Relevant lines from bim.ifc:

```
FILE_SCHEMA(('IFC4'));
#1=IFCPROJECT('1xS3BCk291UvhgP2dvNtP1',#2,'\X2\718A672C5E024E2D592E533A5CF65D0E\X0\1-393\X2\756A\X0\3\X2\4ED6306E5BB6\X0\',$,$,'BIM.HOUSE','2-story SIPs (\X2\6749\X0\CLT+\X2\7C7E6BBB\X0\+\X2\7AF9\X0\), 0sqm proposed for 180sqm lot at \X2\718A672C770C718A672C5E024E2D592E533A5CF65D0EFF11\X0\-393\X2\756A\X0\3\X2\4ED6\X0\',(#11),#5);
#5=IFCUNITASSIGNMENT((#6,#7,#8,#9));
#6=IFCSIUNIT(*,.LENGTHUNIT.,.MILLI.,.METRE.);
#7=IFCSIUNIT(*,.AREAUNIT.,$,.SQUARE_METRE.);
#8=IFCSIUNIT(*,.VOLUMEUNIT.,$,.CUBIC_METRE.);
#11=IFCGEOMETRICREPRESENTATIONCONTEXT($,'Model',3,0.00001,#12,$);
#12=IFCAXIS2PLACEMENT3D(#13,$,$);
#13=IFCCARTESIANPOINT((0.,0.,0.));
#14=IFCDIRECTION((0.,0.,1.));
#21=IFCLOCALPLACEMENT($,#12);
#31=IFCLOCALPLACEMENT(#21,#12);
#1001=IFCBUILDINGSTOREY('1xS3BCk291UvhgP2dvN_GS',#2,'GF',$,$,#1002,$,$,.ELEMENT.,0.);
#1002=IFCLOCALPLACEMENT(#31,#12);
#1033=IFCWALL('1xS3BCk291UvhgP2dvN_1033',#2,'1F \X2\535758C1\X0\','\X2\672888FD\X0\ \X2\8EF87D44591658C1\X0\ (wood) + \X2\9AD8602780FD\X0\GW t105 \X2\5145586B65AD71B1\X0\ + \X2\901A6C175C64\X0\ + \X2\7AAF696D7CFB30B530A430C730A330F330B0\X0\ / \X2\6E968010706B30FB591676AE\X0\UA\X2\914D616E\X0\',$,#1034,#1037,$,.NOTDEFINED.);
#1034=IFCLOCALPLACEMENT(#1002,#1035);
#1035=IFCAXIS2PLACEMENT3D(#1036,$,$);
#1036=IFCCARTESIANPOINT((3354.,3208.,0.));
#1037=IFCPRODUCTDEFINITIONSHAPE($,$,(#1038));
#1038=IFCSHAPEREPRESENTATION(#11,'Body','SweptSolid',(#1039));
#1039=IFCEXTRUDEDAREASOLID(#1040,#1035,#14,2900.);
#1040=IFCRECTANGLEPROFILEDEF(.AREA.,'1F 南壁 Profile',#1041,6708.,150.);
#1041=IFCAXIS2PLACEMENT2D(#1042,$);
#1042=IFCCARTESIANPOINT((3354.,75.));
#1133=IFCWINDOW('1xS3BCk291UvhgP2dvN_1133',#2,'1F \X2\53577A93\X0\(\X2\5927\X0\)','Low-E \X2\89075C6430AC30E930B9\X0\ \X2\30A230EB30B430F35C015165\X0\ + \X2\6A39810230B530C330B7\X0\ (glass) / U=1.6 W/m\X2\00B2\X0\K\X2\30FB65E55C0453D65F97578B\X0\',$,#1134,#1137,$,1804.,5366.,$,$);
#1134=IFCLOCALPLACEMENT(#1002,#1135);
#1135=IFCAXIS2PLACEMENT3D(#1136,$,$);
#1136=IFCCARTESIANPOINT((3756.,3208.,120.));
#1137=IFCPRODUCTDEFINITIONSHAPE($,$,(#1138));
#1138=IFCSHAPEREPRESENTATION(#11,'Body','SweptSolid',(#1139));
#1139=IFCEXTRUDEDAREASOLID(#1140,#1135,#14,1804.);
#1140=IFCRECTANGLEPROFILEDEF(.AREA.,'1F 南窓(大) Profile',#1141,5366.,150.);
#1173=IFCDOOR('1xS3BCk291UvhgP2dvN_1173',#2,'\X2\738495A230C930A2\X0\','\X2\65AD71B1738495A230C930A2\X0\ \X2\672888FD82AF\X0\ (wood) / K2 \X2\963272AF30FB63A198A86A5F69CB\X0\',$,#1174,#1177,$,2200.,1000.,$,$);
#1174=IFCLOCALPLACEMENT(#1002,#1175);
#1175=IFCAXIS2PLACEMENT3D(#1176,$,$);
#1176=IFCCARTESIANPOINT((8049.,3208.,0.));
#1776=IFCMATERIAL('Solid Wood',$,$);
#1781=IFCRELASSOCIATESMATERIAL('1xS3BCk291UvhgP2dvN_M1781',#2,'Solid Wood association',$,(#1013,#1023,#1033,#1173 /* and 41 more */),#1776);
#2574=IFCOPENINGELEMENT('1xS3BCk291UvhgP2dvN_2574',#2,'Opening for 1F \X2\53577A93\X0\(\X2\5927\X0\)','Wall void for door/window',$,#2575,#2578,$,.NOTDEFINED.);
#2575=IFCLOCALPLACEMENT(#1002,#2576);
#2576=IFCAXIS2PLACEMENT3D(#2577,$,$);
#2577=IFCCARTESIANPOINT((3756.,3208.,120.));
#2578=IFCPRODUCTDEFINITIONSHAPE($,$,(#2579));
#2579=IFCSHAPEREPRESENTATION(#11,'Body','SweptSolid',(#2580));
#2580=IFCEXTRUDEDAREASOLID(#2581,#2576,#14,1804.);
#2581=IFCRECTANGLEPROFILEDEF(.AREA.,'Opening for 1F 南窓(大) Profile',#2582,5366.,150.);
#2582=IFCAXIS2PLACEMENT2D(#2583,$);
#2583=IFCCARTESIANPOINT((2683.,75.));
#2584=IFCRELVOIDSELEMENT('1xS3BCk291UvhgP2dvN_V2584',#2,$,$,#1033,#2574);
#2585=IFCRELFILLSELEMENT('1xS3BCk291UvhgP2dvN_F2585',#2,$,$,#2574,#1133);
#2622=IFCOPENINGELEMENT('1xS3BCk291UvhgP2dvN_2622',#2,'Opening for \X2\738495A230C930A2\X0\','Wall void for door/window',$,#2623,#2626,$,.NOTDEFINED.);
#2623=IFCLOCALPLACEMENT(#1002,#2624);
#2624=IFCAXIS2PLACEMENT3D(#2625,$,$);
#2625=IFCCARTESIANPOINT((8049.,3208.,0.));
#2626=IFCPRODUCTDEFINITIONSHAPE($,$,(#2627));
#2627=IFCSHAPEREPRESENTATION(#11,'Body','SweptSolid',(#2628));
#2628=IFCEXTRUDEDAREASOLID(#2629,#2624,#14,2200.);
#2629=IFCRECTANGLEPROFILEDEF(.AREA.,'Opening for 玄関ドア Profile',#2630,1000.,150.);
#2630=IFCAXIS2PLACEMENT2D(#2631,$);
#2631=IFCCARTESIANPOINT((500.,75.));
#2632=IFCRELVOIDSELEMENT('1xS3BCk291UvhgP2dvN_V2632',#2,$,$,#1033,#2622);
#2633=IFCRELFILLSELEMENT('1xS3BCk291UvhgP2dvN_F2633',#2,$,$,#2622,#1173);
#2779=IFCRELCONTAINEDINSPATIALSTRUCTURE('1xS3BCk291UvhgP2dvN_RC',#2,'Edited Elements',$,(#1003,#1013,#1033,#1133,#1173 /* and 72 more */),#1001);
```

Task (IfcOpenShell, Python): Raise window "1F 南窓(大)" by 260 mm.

```python
import numpy as np
import ifcopenshell
import ifcopenshell.api.geometry
import ifcopenshell.util.placement
import ifcopenshell.util.unit

model = ifcopenshell.open("bim.ifc")
unit_scale = ifcopenshell.util.unit.calculate_unit_scale(model)

window = model.by_guid("1xS3BCk291UvhgP2dvN_1133")
opening = window.FillsVoids[0].RelatingOpeningElement
dz = 0.26 / unit_scale

shift = np.array([0.0, 0.0, dz])
# The window is not placed relative to its opening, so move both.
for product in (opening, window):
    matrix = ifcopenshell.util.placement.get_local_placement(product.ObjectPlacement)
    matrix[:3, 3] += shift
    ifcopenshell.api.geometry.edit_object_placement(model, product=product, matrix=matrix, is_si=False)

print(f"moved by {dz * unit_scale:+.3f} m")

model.write("bim-out.ifc")
```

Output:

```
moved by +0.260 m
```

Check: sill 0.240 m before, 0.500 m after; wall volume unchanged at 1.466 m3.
